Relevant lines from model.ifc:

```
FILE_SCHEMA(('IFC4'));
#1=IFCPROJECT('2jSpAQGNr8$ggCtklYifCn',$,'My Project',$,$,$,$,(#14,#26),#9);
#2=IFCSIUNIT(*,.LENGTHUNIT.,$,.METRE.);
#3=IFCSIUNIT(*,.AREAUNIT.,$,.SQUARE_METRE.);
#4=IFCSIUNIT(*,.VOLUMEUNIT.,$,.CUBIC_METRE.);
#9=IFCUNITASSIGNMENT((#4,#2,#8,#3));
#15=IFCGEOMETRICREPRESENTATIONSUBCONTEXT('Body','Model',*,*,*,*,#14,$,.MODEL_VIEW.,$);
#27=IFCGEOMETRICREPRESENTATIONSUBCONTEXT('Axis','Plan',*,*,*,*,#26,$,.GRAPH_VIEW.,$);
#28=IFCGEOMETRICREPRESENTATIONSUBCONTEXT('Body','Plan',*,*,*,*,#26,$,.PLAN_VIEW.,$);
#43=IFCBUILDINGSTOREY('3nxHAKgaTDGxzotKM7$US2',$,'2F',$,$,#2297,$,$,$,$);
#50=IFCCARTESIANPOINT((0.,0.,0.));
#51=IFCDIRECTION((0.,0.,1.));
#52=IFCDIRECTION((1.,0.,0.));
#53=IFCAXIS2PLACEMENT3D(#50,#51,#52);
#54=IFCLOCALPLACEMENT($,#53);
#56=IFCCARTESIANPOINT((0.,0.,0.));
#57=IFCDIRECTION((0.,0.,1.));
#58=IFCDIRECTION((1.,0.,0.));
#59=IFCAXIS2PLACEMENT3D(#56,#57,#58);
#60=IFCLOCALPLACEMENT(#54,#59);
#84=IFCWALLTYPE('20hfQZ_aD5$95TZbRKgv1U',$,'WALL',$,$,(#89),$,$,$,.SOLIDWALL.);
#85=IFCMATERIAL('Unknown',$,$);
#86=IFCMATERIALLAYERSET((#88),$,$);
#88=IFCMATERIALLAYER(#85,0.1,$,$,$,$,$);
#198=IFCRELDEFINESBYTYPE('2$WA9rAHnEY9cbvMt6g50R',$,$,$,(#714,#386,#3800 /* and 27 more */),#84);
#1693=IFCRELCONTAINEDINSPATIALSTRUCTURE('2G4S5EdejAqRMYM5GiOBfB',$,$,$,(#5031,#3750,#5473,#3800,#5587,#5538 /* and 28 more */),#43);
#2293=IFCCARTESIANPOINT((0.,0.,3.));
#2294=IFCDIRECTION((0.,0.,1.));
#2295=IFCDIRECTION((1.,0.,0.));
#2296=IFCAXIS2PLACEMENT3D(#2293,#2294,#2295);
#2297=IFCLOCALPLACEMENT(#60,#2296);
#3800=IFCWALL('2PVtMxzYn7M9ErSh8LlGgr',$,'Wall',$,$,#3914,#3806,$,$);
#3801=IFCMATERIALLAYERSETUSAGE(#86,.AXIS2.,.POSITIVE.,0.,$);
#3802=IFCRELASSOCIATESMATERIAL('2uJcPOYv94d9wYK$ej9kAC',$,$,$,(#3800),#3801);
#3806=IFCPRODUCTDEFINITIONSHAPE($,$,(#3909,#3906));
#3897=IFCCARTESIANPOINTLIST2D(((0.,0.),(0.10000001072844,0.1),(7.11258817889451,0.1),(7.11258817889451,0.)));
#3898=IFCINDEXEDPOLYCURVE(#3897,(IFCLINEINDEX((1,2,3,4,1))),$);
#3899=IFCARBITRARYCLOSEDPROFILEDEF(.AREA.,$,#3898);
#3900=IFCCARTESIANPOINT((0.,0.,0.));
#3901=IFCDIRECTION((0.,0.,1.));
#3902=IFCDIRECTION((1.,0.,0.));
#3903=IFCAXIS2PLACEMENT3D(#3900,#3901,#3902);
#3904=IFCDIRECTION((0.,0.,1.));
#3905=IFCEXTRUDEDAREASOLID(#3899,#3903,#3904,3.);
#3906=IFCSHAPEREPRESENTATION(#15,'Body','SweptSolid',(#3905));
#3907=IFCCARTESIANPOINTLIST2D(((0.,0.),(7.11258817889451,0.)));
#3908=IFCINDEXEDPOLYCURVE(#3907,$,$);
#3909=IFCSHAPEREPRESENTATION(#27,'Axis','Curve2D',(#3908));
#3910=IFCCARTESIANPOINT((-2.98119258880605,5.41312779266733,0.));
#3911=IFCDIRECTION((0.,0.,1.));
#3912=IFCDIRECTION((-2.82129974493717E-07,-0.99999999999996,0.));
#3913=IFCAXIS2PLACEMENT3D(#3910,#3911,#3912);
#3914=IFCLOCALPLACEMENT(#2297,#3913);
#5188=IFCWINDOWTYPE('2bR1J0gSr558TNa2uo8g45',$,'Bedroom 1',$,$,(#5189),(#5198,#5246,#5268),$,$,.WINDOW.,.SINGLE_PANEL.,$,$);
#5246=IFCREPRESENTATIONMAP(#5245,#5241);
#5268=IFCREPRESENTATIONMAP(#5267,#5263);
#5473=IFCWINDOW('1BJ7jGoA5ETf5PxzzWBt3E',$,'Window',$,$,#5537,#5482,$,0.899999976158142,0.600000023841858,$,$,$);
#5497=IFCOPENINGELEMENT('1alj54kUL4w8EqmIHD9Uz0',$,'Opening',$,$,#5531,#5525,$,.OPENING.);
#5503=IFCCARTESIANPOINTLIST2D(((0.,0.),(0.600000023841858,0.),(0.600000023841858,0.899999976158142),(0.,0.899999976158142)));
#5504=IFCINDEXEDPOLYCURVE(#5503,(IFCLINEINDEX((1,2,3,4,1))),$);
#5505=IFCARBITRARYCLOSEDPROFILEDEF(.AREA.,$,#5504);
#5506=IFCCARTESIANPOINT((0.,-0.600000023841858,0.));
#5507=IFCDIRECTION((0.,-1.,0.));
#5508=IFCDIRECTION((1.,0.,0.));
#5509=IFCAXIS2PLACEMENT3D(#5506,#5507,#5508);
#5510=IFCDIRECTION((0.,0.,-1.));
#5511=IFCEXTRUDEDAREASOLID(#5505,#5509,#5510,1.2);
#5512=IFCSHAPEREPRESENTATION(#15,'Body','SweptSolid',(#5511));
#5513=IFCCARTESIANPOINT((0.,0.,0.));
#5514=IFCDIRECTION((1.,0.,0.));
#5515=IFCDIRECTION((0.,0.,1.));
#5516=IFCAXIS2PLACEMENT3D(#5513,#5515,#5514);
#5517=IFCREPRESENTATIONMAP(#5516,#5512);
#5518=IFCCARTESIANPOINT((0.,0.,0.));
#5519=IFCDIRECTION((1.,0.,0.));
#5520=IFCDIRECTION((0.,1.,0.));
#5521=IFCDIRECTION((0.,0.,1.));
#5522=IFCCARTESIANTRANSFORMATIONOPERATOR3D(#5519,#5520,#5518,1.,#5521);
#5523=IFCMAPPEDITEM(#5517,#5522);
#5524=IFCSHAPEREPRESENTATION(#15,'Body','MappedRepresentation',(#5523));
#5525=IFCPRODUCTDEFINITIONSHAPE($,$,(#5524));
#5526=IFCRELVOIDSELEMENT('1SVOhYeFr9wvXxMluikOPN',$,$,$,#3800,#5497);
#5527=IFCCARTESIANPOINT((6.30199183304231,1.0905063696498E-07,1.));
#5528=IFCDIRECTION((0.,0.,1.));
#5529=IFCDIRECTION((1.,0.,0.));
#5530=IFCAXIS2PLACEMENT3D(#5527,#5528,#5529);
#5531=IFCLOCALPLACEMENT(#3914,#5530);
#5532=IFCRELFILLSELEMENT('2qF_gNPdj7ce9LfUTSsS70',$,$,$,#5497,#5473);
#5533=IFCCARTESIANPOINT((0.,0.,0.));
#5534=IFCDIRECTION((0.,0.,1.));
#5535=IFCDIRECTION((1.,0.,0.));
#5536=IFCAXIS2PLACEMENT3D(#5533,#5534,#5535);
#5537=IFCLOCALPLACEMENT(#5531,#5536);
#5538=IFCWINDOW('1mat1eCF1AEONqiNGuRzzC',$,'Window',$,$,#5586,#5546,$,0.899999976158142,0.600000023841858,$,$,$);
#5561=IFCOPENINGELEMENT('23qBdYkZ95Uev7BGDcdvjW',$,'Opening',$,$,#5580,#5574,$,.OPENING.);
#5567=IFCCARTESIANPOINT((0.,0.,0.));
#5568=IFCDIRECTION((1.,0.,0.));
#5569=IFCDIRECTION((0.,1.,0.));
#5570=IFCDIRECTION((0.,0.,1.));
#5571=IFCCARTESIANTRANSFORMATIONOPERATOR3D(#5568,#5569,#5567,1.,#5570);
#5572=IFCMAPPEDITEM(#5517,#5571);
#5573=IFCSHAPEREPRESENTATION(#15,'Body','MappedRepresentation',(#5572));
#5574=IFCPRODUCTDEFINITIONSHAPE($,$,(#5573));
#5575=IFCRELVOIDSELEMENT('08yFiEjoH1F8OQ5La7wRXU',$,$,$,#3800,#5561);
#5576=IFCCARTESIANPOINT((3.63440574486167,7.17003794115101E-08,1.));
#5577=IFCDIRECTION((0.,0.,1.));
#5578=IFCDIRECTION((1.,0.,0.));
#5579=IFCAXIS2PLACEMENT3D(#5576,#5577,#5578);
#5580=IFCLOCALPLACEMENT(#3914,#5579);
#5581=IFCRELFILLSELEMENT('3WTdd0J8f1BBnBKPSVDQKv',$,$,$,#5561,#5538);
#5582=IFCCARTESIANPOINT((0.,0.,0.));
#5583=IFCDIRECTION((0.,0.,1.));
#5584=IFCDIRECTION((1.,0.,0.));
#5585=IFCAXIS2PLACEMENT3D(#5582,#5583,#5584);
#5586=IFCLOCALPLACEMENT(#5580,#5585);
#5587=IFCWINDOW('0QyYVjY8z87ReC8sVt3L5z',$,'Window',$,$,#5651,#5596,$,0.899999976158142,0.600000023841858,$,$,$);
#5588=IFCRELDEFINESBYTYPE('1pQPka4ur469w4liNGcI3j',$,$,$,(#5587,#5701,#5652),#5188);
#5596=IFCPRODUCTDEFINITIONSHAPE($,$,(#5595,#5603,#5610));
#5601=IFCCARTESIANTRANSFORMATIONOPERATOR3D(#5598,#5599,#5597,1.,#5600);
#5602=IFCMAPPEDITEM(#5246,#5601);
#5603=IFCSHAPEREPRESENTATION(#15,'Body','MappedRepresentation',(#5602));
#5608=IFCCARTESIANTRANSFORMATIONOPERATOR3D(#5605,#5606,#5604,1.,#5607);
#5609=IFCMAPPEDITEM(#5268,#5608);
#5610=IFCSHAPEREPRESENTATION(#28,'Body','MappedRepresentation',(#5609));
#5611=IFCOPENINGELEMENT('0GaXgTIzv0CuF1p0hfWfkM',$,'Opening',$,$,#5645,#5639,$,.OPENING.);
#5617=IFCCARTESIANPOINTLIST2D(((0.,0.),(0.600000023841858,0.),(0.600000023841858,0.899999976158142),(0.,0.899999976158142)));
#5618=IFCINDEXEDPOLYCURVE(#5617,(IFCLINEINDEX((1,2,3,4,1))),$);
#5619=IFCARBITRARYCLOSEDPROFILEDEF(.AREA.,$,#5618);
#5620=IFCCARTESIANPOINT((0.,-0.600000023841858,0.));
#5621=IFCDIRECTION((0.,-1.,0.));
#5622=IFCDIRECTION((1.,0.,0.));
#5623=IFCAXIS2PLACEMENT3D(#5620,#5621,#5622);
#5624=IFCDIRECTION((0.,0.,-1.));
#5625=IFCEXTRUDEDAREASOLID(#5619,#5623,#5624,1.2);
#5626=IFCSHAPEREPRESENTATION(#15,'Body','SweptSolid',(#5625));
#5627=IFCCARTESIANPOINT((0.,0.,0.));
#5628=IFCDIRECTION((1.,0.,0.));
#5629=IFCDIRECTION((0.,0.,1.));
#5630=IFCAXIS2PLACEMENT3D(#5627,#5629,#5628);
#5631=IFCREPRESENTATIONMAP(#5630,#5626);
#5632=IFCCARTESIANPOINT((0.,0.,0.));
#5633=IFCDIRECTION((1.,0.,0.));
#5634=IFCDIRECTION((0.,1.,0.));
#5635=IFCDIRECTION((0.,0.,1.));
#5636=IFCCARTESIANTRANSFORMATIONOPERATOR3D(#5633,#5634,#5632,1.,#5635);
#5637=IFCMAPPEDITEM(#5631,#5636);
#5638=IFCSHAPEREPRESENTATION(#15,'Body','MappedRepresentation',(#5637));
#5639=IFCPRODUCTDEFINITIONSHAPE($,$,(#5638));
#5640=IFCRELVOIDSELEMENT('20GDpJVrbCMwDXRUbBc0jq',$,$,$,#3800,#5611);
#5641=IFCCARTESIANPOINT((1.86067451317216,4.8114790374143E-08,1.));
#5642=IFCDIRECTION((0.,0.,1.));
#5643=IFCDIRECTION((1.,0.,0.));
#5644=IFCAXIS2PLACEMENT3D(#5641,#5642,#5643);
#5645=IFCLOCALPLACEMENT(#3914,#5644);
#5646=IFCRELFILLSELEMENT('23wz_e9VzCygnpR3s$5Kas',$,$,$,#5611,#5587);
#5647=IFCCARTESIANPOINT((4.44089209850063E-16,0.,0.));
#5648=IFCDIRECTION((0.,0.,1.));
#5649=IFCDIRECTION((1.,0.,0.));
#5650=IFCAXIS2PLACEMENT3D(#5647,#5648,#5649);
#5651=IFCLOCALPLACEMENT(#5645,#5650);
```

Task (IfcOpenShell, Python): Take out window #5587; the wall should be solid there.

```python
import ifcopenshell
import ifcopenshell.api.feature
import ifcopenshell.api.root
import ifcopenshell.geom
import ifcopenshell.util.shape

model = ifcopenshell.open("model.ifc")
settings = ifcopenshell.geom.settings()


def volume(element):
    """Net volume in cubic metres, openings subtracted."""
    shape = ifcopenshell.geom.create_shape(settings, element)
    return ifcopenshell.util.shape.get_volume(shape.geometry)


window = model.by_id(5587)
opening = window.FillsVoids[0].RelatingOpeningElement
wall = opening.VoidsElements[0].RelatingBuildingElement
before = volume(wall)

ifcopenshell.api.root.remove_product(model, product=window)
ifcopenshell.api.feature.remove_feature(model, feature=opening)

after = volume(wall)

print(f"wall volume {before:.3f} -> {after:.3f} m3")

model.write("model-out.ifc")
```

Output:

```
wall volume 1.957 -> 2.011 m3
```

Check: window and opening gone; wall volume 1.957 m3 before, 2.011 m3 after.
